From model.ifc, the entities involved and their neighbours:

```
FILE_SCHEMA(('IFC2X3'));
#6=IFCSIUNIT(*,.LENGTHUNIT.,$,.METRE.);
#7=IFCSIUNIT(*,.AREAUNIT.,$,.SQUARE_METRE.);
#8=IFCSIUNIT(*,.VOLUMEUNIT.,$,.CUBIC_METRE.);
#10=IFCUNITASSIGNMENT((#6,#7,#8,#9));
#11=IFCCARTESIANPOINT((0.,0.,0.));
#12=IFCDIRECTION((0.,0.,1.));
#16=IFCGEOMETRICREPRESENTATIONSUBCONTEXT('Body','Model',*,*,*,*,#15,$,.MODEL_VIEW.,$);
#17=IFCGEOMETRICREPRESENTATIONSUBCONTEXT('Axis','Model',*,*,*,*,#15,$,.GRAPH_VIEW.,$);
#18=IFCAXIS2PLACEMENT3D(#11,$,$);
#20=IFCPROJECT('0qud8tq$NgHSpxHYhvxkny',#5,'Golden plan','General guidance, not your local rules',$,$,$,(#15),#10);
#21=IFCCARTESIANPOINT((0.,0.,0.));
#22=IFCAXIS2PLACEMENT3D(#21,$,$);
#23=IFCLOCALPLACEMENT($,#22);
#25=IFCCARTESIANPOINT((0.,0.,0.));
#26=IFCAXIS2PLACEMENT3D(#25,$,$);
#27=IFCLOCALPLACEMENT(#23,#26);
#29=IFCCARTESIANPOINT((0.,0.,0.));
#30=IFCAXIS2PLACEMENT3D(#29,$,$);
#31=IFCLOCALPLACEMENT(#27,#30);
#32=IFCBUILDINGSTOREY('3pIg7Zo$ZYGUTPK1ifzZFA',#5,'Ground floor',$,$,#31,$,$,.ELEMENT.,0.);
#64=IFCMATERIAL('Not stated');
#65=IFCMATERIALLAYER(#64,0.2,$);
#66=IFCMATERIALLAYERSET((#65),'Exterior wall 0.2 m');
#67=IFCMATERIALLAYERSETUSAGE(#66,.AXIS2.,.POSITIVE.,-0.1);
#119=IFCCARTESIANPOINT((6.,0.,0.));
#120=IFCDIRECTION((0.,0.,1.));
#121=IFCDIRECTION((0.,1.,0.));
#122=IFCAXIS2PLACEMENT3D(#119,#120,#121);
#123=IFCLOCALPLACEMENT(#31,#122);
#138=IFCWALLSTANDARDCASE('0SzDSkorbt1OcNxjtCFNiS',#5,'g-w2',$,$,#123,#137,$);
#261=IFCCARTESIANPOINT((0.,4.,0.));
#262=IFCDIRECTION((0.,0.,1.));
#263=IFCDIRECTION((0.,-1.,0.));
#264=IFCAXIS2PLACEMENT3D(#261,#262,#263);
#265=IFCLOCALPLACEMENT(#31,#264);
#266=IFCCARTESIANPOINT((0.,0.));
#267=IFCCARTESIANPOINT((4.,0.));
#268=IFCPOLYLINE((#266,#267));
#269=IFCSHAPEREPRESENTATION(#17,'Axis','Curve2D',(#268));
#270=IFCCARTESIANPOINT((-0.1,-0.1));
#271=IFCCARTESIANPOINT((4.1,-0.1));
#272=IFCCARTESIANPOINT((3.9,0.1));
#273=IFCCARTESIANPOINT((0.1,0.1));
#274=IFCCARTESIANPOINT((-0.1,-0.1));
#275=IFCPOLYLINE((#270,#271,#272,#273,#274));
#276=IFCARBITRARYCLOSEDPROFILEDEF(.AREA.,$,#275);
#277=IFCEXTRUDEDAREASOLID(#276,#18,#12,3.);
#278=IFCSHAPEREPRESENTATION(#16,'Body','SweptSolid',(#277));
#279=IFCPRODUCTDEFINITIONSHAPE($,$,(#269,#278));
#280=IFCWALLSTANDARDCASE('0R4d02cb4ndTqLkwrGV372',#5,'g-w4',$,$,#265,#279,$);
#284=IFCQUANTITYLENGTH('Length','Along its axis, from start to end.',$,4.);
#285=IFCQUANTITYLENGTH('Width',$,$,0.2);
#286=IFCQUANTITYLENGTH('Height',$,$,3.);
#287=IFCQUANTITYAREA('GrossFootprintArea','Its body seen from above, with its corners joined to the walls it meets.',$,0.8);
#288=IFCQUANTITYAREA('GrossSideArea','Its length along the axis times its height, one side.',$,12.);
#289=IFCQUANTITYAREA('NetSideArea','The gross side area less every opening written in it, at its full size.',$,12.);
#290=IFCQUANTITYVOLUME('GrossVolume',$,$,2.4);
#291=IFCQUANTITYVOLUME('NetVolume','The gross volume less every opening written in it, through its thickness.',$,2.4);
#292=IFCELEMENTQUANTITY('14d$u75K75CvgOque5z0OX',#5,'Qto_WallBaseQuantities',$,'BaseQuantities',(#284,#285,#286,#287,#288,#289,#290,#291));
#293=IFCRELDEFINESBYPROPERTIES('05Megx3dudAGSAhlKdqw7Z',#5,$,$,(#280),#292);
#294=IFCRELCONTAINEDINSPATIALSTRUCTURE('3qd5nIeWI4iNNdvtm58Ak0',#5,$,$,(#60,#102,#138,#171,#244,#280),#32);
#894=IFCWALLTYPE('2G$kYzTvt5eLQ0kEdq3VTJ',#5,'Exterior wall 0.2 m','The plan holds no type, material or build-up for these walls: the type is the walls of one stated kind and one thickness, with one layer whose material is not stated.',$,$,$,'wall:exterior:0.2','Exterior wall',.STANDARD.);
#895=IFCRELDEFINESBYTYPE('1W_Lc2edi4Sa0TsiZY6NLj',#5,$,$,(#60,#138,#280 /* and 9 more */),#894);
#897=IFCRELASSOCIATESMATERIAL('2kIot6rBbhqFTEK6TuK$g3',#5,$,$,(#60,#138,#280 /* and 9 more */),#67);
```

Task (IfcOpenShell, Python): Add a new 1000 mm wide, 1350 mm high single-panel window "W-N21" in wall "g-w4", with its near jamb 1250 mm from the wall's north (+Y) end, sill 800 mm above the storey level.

```python
import numpy as np
import ifcopenshell
import ifcopenshell.api.feature
import ifcopenshell.api.geometry
import ifcopenshell.api.pset
import ifcopenshell.api.root
import ifcopenshell.api.spatial
import ifcopenshell.api.type
import ifcopenshell.geom
import ifcopenshell.util.element
import ifcopenshell.util.placement
import ifcopenshell.util.representation
import ifcopenshell.util.shape
import ifcopenshell.util.unit

model = ifcopenshell.open("model.ifc")
unit_scale = ifcopenshell.util.unit.calculate_unit_scale(model)
area_scale = ifcopenshell.util.unit.calculate_unit_scale(model, "AREAUNIT")
volume_scale = ifcopenshell.util.unit.calculate_unit_scale(model, "VOLUMEUNIT")
settings = ifcopenshell.geom.settings()


def volume(element):
    """Net volume in cubic metres, openings subtracted."""
    shape = ifcopenshell.geom.create_shape(settings, element)
    return ifcopenshell.util.shape.get_volume(shape.geometry)


wall = model.by_guid("0R4d02cb4ndTqLkwrGV372")
storey = ifcopenshell.util.element.get_container(wall, ifc_class="IfcBuildingStorey")
context = ifcopenshell.util.representation.get_context(model, "Model", "Body", "MODEL_VIEW")
before = volume(wall)

width, height, from_end, sill = 1, 1.35, 1.25, 0.8  # metres

# The wall runs along its own X axis, and the end named is its -X end.
wall_shape = ifcopenshell.geom.create_shape(settings, wall)
x, y, z = ifcopenshell.util.shape.get_vertices(wall_shape.geometry).T
start = x.min() + from_end
face, thickness = float(y.min()), float(y.max() - y.min())
wall_matrix = ifcopenshell.util.placement.get_local_placement(wall.ObjectPlacement)
level = ifcopenshell.util.placement.get_local_placement(storey.ObjectPlacement)[2, 3]


def in_wall(x, y):
    """Placement at x, y metres in the wall's axes, at sill height."""
    matrix = wall_matrix.copy()
    matrix[:, 3] = wall_matrix @ np.array([x / unit_scale, y / unit_scale, 0.0, 1.0])
    matrix[2, 3] = level + sill / unit_scale
    return matrix


# Opening: a box that overshoots both wall faces by 50 mm.
opening = ifcopenshell.api.root.create_entity(model, ifc_class="IfcOpeningElement")
box = ifcopenshell.api.geometry.add_wall_representation(
    model, context=context, length=width, height=height, thickness=thickness + 0.1
)
ifcopenshell.api.geometry.assign_representation(model, product=opening, representation=box)
ifcopenshell.api.geometry.edit_object_placement(model, product=opening, matrix=in_wall(start, face - 0.05), is_si=False)
ifcopenshell.api.feature.add_feature(model, feature=opening, element=wall)

window = ifcopenshell.api.root.create_entity(model, ifc_class="IfcWindow", name="W-N21")
window.OverallWidth, window.OverallHeight = width / unit_scale, height / unit_scale
body = ifcopenshell.api.geometry.add_window_representation(
    model,
    context=context,
    overall_width=window.OverallWidth,
    overall_height=window.OverallHeight,
    partition_type="SINGLE_PANEL",
)
ifcopenshell.api.geometry.assign_representation(model, product=window, representation=body)
ifcopenshell.api.spatial.assign_container(model, products=[window], relating_structure=storey)
fills = ifcopenshell.api.feature.add_filling(model, opening=opening, element=window)
fills.OwnerHistory = window.OwnerHistory  # required in IFC2X3

# IFC2X3 keeps the operation on the window style.
style = ifcopenshell.api.root.create_entity(model, ifc_class="IfcWindowStyle", name="W-N21")
style.OperationType, style.ConstructionType = "SINGLE_PANEL", "NOTDEFINED"
style.ParameterTakesPrecedence = style.Sizeable = False
ifcopenshell.api.type.assign_type(model, related_objects=[window], relating_type=style)

# Centre the window in the wall's thickness.
ifcopenshell.api.geometry.edit_object_placement(model, product=window, matrix=in_wall(start, face), is_si=False)
window_shape = ifcopenshell.geom.create_shape(settings, window)
depth = ifcopenshell.util.shape.get_vertices(window_shape.geometry)[:, 1]
offset = face + thickness / 2 - (depth.min() + depth.max()) / 2
ifcopenshell.api.geometry.edit_object_placement(model, product=window, matrix=in_wall(start, offset), is_si=False)

after = volume(wall)

# Update the wall's stored quantities.
qto = model.by_id(ifcopenshell.util.element.get_pset(wall, "Qto_WallBaseQuantities", should_inherit=False)["id"])
ifcopenshell.api.pset.edit_qto(model, qto=qto, properties={
    "NetSideArea": after / thickness / area_scale,
    "NetVolume": after / volume_scale,
})

print(f"wall volume {before:.3f} -> {after:.3f} m3")

model.write("model_edited.ifc")
```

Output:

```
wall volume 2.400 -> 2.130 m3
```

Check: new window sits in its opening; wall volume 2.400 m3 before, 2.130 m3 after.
